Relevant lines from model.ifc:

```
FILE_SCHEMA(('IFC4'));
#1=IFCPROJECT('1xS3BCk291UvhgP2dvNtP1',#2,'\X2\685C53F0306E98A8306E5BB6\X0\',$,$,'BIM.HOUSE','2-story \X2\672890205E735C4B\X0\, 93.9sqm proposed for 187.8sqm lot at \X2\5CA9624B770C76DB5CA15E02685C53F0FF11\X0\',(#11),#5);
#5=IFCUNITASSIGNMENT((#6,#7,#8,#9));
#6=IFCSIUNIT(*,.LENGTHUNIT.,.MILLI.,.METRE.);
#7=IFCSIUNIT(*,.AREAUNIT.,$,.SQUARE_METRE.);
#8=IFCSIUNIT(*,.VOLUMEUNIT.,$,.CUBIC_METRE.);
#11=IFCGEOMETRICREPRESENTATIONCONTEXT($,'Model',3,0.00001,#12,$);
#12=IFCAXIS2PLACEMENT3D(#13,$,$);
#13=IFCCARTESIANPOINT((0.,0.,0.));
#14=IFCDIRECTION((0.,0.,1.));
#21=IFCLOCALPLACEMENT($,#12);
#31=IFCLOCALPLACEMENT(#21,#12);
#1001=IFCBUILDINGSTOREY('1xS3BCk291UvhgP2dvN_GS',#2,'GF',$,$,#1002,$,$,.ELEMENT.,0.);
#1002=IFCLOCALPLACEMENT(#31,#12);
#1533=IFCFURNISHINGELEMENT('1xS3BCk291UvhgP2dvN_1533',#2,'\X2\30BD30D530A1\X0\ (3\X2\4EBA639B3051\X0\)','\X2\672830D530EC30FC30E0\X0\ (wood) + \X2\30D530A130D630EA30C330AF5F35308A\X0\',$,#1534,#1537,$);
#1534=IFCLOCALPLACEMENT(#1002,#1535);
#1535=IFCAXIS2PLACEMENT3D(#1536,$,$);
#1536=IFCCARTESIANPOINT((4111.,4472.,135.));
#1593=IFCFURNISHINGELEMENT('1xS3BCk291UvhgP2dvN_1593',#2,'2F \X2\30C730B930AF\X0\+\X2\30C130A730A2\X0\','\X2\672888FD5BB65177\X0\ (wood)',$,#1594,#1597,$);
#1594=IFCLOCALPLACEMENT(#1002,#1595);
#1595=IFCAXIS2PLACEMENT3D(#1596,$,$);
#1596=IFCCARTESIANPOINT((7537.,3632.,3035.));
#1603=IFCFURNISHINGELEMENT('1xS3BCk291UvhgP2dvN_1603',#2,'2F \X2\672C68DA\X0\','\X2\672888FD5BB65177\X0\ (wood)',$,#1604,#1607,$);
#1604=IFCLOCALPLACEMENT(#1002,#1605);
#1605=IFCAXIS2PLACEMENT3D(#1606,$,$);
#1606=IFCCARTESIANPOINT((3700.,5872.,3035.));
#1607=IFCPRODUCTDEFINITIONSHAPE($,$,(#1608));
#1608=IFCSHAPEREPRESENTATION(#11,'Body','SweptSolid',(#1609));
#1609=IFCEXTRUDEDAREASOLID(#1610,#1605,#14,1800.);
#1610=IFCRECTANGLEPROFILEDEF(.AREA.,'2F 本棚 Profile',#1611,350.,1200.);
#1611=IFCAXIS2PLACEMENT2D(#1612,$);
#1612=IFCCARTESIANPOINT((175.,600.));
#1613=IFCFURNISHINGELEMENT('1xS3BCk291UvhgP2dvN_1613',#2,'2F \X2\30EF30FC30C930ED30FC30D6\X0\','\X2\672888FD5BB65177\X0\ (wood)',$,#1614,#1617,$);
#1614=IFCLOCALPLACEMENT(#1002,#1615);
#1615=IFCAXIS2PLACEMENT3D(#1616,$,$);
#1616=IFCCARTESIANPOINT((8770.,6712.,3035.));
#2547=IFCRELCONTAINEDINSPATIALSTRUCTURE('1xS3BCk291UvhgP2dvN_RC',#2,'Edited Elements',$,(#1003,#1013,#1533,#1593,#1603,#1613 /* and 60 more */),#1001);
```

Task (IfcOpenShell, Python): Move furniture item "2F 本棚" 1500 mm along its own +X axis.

```python
import ifcopenshell
import ifcopenshell.api.geometry
import ifcopenshell.util.placement

model = ifcopenshell.open("model.ifc")

item = model.by_guid("1xS3BCk291UvhgP2dvN_1603")
matrix = ifcopenshell.util.placement.get_local_placement(item.ObjectPlacement)
matrix[:3, 3] += matrix[:3, 0] * 1500.0
ifcopenshell.api.geometry.edit_object_placement(model, product=item, matrix=matrix, is_si=False)

print(ifcopenshell.util.placement.get_local_placement(item.ObjectPlacement).round(3) + 0.0)

model.write("model_updated.ifc")
```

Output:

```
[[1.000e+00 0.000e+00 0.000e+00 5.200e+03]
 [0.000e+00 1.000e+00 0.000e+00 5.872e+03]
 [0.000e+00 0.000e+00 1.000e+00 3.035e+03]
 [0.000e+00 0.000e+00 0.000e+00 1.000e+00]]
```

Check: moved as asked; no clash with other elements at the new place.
